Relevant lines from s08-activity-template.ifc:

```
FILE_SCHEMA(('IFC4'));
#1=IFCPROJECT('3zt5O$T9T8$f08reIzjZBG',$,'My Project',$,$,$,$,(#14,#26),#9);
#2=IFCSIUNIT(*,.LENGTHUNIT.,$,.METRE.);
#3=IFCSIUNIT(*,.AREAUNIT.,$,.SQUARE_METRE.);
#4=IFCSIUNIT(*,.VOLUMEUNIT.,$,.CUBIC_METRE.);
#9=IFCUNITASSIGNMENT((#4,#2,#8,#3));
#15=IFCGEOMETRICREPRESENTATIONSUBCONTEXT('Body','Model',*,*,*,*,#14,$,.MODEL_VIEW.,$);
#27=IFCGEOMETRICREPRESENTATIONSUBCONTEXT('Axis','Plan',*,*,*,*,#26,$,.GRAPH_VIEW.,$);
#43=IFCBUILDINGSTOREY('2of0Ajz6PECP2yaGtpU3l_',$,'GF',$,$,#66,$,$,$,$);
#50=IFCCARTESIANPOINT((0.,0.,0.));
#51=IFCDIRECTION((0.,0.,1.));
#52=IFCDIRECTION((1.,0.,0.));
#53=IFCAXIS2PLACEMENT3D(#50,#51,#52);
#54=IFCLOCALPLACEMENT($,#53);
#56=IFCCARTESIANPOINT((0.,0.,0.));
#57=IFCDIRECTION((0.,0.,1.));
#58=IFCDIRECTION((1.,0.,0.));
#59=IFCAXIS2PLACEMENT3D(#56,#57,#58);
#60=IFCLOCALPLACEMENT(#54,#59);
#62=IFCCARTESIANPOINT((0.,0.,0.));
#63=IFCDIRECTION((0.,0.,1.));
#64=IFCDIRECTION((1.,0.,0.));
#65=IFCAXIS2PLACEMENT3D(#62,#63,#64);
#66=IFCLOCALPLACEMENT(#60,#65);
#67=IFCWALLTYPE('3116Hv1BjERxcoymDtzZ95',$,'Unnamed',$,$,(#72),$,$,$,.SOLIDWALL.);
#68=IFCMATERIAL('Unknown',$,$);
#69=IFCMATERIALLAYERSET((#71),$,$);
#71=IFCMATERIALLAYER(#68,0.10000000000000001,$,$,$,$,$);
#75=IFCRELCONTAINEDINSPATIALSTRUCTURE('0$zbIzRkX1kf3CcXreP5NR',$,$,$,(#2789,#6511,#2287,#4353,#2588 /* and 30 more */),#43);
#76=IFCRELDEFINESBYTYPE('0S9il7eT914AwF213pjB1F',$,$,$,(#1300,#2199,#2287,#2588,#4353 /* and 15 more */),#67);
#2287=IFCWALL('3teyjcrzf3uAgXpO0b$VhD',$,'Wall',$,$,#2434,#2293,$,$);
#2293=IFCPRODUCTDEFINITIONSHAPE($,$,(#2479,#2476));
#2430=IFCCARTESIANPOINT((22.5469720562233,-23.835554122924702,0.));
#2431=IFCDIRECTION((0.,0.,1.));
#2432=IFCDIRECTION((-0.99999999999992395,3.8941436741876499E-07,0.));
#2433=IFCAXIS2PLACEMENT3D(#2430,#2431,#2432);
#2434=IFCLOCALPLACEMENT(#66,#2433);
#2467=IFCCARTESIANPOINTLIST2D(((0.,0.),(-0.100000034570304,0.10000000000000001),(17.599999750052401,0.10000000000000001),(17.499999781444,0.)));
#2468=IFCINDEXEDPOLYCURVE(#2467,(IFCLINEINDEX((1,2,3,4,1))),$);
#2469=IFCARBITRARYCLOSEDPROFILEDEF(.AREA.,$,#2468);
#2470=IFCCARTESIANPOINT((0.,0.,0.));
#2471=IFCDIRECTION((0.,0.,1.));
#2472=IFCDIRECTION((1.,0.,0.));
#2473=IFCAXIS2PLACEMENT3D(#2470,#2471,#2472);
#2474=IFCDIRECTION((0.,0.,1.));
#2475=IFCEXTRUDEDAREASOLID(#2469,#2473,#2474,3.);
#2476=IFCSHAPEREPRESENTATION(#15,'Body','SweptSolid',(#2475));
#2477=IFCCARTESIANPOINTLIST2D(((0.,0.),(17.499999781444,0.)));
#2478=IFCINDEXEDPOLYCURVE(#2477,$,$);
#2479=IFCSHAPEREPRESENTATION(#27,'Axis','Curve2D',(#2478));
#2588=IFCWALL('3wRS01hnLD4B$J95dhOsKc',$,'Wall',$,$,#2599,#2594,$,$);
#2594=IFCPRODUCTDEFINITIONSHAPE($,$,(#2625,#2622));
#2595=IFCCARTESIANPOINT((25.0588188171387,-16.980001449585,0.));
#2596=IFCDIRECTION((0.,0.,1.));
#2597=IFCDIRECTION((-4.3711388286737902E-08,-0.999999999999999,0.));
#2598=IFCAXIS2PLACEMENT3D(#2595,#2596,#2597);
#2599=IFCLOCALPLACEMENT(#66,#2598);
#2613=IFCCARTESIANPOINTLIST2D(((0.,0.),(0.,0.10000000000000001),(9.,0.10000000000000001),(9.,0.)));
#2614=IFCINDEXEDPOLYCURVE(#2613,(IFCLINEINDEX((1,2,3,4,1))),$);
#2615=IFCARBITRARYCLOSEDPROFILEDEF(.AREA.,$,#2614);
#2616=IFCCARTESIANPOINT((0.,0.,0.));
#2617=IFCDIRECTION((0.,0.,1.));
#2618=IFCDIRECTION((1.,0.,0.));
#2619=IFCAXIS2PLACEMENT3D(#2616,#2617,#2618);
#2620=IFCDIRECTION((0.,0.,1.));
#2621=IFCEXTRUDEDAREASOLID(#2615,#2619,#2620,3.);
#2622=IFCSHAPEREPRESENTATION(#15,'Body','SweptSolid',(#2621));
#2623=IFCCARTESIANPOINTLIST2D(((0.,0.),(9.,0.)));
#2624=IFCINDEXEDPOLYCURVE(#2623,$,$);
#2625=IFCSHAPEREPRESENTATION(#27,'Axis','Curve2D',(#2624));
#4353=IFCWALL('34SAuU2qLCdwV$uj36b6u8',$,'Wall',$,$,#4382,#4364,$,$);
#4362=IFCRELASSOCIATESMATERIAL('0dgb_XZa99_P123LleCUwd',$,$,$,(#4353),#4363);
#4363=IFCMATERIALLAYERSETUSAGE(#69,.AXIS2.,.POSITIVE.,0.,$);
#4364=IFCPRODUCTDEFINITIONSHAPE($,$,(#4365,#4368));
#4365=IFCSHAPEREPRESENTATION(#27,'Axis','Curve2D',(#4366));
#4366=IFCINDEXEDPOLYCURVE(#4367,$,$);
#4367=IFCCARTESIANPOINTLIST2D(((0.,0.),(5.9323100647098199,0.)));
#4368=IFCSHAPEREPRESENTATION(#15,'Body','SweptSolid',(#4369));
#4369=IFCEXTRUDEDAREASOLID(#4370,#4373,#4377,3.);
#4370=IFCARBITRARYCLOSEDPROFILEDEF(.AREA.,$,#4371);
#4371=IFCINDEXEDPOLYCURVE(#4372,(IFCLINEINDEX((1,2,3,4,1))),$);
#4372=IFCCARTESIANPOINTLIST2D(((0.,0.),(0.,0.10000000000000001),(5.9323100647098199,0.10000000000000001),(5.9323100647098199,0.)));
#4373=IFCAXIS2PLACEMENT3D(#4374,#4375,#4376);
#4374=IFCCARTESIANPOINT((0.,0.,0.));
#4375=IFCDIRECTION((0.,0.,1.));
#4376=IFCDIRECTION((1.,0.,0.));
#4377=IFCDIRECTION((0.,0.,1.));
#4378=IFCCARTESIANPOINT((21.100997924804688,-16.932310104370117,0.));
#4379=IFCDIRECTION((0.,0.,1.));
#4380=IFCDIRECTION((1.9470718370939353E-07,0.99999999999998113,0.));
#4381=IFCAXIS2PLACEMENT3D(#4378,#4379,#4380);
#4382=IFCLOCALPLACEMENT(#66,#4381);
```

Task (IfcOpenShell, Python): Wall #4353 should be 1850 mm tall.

```python
import ifcopenshell
import ifcopenshell.geom
import ifcopenshell.util.representation
import ifcopenshell.util.shape

model = ifcopenshell.open("s08-activity-template.ifc")
settings = ifcopenshell.geom.settings()


def volume(element):
    """Net volume in cubic metres, openings subtracted."""
    shape = ifcopenshell.geom.create_shape(settings, element)
    return ifcopenshell.util.shape.get_volume(shape.geometry)


wall = model.by_id(4353)
before = volume(wall)

body = ifcopenshell.util.representation.get_representation(wall, "Model", "Body")
solid = body.Items[0]
old_height = solid.Depth
solid.Depth = 1.85
after = volume(wall)

print(f"height {old_height:g} -> {solid.Depth:g}, volume {before:.3f} -> {after:.3f} m3")

model.write("s08-activity-template_updated.ifc")
```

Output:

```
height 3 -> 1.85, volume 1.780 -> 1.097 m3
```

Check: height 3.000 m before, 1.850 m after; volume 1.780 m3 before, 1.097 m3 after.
